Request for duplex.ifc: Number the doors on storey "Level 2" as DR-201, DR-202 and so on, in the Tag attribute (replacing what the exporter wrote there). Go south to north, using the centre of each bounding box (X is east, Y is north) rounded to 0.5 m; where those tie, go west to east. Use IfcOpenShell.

First a look at what the model holds.

```python
import ifcopenshell
import ifcopenshell.util.element
import ifcopenshell.util.placement

model = ifcopenshell.open("duplex.ifc")
print(model.schema)
storey = next(s for s in model.by_type("IfcBuildingStorey") if s.Name == "Level 2")
doors = [e for e in ifcopenshell.util.element.get_decomposition(storey) if e.is_a("IfcDoor")]
for e in sorted(doors, key=lambda e: e.id()):
    origin = ifcopenshell.util.placement.get_local_placement(e.ObjectPlacement)[:3, 3]
    print(e.id(), e.Tag, e.Name, origin.round(2) + 0.0, sep=" | ")
```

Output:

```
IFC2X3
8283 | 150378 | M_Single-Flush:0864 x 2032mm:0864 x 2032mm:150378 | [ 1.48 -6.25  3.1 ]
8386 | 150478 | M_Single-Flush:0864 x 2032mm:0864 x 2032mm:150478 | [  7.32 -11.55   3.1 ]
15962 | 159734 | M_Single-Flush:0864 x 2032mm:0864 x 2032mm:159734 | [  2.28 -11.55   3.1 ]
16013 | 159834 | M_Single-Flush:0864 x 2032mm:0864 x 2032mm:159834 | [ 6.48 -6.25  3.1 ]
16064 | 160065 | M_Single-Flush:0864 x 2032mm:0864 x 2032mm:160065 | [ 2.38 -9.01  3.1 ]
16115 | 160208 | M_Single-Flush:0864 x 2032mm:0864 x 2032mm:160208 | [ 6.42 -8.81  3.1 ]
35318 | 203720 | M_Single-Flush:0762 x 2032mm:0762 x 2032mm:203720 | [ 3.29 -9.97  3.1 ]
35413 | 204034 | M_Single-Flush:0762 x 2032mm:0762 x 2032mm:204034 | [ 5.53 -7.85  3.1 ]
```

```python
import ifcopenshell
import ifcopenshell.geom
import ifcopenshell.util.element
import ifcopenshell.util.shape

model = ifcopenshell.open("duplex.ifc")
settings = ifcopenshell.geom.settings()
settings.set("use-world-coords", True)


def centre(element):
    shape = ifcopenshell.geom.create_shape(settings, element)
    return ifcopenshell.util.shape.get_bbox_centroid(shape.geometry)


storey = next(s for s in model.by_type("IfcBuildingStorey") if s.Name == "Level 2")
doors = [e for e in ifcopenshell.util.element.get_decomposition(storey) if e.is_a("IfcDoor")]

# Insertion points can sit at a corner or the storey origin, so sort by the geometry (in metres).
centres = {e: centre(e) for e in doors}
doors.sort(key=lambda e: (round(centres[e][1] / 0.5), centres[e][0]))

for i, e in enumerate(doors, start=1):
    number = f"DR-2{i:02d}"
    e.Tag = number
    print(e.id(), number)

model.write("duplex-out.ifc")
```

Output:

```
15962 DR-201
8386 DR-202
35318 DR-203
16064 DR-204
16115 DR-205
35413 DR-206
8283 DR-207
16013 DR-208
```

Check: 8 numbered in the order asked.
